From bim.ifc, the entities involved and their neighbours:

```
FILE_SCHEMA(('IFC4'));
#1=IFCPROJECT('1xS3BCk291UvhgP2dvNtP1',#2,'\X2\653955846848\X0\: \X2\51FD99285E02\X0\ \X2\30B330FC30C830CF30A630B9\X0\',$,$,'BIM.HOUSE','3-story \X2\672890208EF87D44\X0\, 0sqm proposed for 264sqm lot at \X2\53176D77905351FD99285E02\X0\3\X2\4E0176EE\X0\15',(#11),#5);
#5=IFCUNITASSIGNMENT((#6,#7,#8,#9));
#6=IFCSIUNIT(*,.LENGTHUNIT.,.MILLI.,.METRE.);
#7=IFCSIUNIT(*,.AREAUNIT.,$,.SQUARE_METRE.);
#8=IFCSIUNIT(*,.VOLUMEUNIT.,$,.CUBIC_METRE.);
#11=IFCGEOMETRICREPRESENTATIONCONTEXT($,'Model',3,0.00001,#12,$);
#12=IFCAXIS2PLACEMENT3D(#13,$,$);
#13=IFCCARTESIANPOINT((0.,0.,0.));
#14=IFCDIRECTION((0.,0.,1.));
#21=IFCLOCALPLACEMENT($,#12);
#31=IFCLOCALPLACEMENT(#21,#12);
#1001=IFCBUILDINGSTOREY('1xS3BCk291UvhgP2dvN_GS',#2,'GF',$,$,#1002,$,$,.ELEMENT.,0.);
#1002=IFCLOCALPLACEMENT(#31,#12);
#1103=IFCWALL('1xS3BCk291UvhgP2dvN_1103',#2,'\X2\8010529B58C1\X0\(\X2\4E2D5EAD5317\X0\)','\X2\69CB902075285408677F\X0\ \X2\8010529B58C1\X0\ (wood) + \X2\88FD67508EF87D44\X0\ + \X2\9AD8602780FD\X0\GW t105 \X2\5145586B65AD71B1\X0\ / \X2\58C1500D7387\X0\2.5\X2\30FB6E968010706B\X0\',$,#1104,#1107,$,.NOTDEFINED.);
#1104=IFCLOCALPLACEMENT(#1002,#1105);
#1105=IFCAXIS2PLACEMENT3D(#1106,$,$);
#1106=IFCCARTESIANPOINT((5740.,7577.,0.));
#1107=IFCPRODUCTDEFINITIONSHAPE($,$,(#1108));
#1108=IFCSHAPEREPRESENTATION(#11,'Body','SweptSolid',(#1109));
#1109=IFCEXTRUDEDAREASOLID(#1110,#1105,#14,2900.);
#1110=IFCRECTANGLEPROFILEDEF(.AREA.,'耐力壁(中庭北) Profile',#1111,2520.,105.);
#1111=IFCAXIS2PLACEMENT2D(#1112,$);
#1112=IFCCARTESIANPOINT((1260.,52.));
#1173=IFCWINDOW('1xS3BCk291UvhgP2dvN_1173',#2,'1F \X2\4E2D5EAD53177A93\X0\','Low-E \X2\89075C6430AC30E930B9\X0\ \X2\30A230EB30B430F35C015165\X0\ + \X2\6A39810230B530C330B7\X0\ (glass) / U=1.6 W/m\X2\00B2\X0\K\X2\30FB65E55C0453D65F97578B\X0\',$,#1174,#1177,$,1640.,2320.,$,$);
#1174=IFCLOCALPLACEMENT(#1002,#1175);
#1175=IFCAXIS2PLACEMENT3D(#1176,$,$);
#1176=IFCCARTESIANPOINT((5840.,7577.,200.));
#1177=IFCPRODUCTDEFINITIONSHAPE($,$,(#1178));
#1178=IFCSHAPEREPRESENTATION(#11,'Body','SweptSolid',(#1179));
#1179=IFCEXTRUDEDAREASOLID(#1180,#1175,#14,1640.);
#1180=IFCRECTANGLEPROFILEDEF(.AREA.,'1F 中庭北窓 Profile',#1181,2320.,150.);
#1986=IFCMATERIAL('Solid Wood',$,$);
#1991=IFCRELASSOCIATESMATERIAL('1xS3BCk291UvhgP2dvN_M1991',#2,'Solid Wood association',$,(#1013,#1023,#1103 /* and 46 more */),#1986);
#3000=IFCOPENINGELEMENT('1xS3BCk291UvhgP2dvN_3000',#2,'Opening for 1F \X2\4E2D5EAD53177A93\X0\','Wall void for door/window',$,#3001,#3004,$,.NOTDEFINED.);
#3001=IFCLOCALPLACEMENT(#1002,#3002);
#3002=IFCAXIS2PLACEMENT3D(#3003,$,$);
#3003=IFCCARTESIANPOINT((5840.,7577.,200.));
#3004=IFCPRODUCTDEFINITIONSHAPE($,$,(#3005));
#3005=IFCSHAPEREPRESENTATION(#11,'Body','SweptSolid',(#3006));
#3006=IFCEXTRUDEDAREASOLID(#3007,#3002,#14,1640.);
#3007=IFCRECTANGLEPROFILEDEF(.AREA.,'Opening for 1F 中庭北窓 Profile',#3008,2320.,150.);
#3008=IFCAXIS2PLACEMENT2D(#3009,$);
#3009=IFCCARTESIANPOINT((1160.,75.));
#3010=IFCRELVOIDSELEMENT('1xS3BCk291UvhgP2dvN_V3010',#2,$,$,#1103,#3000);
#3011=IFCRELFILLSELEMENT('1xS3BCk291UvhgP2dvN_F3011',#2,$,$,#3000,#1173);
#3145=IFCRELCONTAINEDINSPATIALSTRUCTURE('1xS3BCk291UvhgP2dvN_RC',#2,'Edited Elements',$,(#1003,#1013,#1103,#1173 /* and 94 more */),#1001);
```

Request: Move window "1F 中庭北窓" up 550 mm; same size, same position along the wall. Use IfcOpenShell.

```python
import numpy as np
import ifcopenshell
import ifcopenshell.api.geometry
import ifcopenshell.util.placement
import ifcopenshell.util.unit

model = ifcopenshell.open("bim.ifc")
unit_scale = ifcopenshell.util.unit.calculate_unit_scale(model)

window = model.by_guid("1xS3BCk291UvhgP2dvN_1173")
opening = window.FillsVoids[0].RelatingOpeningElement
dz = 550.0

shift = np.array([0.0, 0.0, dz])
# The window is not placed relative to its opening, so move both.
for product in (opening, window):
    matrix = ifcopenshell.util.placement.get_local_placement(product.ObjectPlacement)
    matrix[:3, 3] += shift
    ifcopenshell.api.geometry.edit_object_placement(model, product=product, matrix=matrix, is_si=False)

print(f"moved by {dz * unit_scale:+.3f} m")

model.write("bim_rev.ifc")
```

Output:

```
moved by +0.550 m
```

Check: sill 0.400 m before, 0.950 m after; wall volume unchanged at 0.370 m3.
